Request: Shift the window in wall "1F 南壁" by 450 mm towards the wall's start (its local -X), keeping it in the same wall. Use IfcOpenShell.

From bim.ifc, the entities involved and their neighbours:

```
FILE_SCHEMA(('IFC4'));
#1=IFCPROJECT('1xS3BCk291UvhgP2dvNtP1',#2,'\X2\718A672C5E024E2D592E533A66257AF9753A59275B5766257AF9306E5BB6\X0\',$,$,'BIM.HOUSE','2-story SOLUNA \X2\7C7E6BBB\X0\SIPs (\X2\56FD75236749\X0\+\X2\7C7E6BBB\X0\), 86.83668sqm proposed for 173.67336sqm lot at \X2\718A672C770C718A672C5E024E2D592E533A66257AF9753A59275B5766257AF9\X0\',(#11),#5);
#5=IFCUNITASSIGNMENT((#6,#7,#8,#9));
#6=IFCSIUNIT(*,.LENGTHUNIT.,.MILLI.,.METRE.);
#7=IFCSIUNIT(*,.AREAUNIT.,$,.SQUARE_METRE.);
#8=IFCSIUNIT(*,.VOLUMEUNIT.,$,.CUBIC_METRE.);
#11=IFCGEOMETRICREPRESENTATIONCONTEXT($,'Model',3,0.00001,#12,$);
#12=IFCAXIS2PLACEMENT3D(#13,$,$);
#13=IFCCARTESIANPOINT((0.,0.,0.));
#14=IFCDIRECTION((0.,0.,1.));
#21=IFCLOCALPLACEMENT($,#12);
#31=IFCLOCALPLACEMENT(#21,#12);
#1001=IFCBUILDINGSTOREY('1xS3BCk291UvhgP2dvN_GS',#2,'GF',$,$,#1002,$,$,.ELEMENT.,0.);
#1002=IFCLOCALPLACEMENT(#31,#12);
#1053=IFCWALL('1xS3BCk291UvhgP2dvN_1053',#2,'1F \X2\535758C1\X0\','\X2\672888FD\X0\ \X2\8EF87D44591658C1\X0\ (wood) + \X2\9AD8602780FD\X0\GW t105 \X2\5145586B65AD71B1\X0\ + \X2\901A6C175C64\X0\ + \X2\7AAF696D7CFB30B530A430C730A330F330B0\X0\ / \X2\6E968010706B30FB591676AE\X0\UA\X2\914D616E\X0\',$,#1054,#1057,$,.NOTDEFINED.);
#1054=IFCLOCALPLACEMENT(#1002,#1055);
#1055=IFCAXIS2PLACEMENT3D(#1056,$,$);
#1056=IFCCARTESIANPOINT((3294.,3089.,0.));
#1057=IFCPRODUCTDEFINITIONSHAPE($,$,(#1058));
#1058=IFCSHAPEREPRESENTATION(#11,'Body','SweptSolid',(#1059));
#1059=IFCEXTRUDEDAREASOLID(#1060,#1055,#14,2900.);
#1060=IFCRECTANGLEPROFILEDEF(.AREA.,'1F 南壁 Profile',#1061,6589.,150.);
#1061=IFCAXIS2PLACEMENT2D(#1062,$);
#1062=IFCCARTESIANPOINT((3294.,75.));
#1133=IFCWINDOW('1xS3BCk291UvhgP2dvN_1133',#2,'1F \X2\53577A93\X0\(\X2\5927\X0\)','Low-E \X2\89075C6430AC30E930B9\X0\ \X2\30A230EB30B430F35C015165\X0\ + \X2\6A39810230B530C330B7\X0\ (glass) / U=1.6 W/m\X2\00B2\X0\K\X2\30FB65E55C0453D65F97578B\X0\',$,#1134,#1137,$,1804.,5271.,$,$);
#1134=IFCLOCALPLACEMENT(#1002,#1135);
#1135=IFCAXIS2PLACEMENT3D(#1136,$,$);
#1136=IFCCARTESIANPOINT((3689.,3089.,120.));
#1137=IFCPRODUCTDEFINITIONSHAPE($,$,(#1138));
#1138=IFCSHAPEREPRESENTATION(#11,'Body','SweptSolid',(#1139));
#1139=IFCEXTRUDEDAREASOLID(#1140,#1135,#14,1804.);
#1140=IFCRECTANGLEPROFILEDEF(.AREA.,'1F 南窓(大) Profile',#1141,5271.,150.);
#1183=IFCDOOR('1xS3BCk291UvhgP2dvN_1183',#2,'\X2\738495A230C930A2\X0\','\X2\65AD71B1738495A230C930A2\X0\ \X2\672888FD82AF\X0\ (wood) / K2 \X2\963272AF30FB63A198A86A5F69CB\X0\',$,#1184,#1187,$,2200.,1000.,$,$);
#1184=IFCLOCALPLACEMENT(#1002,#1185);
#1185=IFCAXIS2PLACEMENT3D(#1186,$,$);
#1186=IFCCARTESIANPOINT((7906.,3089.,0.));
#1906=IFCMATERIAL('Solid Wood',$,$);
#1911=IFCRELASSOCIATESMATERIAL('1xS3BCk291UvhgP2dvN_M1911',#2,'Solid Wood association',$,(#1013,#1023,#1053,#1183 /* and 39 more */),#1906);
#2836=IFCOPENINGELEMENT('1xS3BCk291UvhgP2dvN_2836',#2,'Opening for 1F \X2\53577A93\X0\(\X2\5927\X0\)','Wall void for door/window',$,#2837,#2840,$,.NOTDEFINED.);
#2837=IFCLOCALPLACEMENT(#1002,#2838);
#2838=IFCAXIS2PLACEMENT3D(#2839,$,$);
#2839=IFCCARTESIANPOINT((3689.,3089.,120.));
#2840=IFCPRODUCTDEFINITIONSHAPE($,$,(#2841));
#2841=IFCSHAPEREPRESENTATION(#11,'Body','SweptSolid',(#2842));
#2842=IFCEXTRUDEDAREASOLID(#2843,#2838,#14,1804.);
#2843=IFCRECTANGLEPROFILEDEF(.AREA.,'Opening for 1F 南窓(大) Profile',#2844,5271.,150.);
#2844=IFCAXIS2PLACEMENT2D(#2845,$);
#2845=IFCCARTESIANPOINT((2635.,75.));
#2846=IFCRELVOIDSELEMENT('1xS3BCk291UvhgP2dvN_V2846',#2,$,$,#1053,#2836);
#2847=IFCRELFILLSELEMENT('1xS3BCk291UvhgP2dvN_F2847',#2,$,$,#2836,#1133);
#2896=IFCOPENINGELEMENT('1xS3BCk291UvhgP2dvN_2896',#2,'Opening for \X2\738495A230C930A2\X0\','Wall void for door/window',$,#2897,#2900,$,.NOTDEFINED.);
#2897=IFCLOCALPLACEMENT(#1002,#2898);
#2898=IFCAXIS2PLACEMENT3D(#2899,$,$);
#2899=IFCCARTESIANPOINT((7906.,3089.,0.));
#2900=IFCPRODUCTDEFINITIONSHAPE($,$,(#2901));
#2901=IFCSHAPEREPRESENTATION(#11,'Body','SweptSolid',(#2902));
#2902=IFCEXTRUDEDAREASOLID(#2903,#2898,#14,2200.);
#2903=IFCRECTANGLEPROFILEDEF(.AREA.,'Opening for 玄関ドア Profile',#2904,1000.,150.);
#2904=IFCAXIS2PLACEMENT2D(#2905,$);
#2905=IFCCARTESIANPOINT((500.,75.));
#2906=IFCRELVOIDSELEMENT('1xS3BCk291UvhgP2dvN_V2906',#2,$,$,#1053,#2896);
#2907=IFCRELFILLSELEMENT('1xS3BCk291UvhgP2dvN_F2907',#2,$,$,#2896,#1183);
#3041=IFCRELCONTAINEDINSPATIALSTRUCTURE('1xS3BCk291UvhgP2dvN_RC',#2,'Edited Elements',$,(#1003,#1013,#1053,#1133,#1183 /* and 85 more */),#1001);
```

```python
import ifcopenshell
import ifcopenshell.api.geometry
import ifcopenshell.util.placement

model = ifcopenshell.open("bim.ifc")

window = model.by_guid("1xS3BCk291UvhgP2dvN_1133")
opening = window.FillsVoids[0].RelatingOpeningElement
wall = opening.VoidsElements[0].RelatingBuildingElement

wall_matrix = ifcopenshell.util.placement.get_local_placement(wall.ObjectPlacement)
shift = wall_matrix[:3, 0] * -450.0
before = ifcopenshell.util.placement.get_local_placement(window.ObjectPlacement)[:3, 3].copy()

# The window is not placed relative to its opening, so move both.
for product in (opening, window):
    matrix = ifcopenshell.util.placement.get_local_placement(product.ObjectPlacement)
    matrix[:3, 3] += shift
    ifcopenshell.api.geometry.edit_object_placement(model, product=product, matrix=matrix, is_si=False)

after = ifcopenshell.util.placement.get_local_placement(window.ObjectPlacement)[:3, 3]
print("window moved by", (after - before).round(3) + 0.0)

model.write("bim_v2.ifc")
```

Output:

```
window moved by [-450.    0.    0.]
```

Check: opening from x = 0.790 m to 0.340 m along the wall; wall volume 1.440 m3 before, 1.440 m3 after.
